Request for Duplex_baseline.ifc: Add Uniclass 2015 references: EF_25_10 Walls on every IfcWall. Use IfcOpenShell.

First a look at what the model holds.

```python
import ifcopenshell

model = ifcopenshell.open("Duplex_baseline.ifc")
print(model.schema)
print("classifications:", [c.Name for c in model.by_type("IfcClassification")])
for ifc_class in ("IfcDoor", "IfcRoof", "IfcStair", "IfcWall", "IfcWindow"):
    print(ifc_class, len(model.by_type(ifc_class)))
```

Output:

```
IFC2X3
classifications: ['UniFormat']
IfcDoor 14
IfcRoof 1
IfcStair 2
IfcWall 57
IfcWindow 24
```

```python
import ifcopenshell
import ifcopenshell.api.classification

model = ifcopenshell.open("Duplex_baseline.ifc")

# IFC2X3 requires Source and Edition and has no link from the project to the system.
system = model.create_entity("IfcClassification", Source="NBS", Edition="2015", Name="Uniclass 2015")

codes = {
    "IfcWall": ("EF_25_10", "Walls"),
}
for ifc_class, (code, name) in codes.items():
    products = model.by_type(ifc_class)
    ifcopenshell.api.classification.add_reference(
        model, products=products, classification=system, identification=code, name=name
    )
    print(code, len(products))

model.write("Duplex_baseline_rev.ifc")
```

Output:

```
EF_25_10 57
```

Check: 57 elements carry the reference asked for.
